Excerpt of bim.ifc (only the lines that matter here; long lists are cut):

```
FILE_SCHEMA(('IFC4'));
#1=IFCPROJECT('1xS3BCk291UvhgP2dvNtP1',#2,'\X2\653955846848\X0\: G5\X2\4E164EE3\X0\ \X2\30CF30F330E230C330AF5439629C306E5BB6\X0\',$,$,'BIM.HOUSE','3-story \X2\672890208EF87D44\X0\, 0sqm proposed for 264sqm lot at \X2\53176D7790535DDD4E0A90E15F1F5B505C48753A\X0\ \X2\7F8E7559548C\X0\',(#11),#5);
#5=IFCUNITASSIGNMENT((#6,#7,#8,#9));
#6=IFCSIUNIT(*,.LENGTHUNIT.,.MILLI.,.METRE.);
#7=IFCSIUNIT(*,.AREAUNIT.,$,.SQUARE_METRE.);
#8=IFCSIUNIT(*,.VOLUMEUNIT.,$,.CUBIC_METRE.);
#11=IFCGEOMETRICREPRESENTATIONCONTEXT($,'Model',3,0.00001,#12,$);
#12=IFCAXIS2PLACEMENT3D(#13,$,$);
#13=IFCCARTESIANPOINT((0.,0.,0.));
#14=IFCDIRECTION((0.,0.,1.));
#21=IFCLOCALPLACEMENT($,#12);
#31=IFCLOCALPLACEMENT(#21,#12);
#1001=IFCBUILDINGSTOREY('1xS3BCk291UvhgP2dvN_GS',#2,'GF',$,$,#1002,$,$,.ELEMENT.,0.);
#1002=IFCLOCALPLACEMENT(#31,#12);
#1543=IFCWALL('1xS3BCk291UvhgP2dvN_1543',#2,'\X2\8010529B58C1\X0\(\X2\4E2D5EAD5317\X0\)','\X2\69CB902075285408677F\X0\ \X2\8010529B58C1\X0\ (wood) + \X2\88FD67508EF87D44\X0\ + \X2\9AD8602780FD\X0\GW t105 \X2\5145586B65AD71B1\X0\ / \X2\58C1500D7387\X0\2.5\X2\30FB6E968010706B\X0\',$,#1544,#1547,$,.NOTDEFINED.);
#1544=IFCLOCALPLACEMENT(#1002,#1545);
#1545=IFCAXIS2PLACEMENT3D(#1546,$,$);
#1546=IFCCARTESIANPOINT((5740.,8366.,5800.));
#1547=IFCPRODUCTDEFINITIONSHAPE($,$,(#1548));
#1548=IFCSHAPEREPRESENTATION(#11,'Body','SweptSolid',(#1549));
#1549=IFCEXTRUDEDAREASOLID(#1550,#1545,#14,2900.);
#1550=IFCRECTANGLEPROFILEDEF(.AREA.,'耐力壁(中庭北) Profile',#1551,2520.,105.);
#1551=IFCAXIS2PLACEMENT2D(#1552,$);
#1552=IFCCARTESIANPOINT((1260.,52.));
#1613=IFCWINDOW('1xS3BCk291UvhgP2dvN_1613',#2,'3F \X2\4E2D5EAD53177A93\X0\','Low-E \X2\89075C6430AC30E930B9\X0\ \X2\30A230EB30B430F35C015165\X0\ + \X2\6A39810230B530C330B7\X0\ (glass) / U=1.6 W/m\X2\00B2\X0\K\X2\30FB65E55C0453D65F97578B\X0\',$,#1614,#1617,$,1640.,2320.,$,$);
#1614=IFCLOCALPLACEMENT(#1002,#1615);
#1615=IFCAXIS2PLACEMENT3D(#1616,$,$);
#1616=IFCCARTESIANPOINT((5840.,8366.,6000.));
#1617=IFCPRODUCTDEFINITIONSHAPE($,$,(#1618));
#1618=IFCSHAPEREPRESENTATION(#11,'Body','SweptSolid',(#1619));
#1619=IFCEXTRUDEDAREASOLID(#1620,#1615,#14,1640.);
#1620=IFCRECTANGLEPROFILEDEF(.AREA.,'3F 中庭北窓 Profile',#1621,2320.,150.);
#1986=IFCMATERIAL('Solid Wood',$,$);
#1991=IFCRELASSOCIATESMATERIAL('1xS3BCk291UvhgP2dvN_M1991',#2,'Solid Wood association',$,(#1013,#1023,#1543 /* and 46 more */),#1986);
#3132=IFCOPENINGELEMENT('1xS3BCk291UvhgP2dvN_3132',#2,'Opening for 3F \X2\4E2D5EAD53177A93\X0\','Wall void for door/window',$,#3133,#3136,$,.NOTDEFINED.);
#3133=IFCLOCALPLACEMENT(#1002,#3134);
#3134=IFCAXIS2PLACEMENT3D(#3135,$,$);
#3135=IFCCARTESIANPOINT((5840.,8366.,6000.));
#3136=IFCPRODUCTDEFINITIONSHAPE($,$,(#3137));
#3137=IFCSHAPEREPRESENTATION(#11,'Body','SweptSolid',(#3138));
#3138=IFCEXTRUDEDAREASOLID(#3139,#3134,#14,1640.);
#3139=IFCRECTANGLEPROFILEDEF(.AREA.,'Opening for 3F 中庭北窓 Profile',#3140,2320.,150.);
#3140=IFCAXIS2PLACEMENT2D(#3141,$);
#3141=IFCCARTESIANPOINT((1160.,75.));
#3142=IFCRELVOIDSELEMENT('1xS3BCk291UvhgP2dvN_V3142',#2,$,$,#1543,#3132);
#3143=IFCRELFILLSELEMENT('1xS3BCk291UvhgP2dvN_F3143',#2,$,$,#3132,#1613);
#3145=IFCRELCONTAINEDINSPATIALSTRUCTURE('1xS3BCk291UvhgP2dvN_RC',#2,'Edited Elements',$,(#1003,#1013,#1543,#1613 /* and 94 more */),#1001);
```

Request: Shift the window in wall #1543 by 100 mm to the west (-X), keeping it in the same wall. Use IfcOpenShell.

```python
import ifcopenshell
import ifcopenshell.api.geometry
import ifcopenshell.util.placement
import ifcopenshell.util.unit

model = ifcopenshell.open("bim.ifc")
unit_scale = ifcopenshell.util.unit.calculate_unit_scale(model)

window = model.by_id(1613)
opening = window.FillsVoids[0].RelatingOpeningElement
wall = opening.VoidsElements[0].RelatingBuildingElement

wall_matrix = ifcopenshell.util.placement.get_local_placement(wall.ObjectPlacement)
shift = wall_matrix[:3, 0] * -0.1 / unit_scale
before = ifcopenshell.util.placement.get_local_placement(window.ObjectPlacement)[:3, 3].copy()

# The window is not placed relative to its opening, so move both.
for product in (opening, window):
    matrix = ifcopenshell.util.placement.get_local_placement(product.ObjectPlacement)
    matrix[:3, 3] += shift
    ifcopenshell.api.geometry.edit_object_placement(model, product=product, matrix=matrix, is_si=False)

after = ifcopenshell.util.placement.get_local_placement(window.ObjectPlacement)[:3, 3]
print("window moved by", (after - before).round(3) + 0.0)

model.write("bim_rev.ifc")
```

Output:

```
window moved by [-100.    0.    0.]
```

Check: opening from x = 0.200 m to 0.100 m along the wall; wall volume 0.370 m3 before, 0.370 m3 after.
